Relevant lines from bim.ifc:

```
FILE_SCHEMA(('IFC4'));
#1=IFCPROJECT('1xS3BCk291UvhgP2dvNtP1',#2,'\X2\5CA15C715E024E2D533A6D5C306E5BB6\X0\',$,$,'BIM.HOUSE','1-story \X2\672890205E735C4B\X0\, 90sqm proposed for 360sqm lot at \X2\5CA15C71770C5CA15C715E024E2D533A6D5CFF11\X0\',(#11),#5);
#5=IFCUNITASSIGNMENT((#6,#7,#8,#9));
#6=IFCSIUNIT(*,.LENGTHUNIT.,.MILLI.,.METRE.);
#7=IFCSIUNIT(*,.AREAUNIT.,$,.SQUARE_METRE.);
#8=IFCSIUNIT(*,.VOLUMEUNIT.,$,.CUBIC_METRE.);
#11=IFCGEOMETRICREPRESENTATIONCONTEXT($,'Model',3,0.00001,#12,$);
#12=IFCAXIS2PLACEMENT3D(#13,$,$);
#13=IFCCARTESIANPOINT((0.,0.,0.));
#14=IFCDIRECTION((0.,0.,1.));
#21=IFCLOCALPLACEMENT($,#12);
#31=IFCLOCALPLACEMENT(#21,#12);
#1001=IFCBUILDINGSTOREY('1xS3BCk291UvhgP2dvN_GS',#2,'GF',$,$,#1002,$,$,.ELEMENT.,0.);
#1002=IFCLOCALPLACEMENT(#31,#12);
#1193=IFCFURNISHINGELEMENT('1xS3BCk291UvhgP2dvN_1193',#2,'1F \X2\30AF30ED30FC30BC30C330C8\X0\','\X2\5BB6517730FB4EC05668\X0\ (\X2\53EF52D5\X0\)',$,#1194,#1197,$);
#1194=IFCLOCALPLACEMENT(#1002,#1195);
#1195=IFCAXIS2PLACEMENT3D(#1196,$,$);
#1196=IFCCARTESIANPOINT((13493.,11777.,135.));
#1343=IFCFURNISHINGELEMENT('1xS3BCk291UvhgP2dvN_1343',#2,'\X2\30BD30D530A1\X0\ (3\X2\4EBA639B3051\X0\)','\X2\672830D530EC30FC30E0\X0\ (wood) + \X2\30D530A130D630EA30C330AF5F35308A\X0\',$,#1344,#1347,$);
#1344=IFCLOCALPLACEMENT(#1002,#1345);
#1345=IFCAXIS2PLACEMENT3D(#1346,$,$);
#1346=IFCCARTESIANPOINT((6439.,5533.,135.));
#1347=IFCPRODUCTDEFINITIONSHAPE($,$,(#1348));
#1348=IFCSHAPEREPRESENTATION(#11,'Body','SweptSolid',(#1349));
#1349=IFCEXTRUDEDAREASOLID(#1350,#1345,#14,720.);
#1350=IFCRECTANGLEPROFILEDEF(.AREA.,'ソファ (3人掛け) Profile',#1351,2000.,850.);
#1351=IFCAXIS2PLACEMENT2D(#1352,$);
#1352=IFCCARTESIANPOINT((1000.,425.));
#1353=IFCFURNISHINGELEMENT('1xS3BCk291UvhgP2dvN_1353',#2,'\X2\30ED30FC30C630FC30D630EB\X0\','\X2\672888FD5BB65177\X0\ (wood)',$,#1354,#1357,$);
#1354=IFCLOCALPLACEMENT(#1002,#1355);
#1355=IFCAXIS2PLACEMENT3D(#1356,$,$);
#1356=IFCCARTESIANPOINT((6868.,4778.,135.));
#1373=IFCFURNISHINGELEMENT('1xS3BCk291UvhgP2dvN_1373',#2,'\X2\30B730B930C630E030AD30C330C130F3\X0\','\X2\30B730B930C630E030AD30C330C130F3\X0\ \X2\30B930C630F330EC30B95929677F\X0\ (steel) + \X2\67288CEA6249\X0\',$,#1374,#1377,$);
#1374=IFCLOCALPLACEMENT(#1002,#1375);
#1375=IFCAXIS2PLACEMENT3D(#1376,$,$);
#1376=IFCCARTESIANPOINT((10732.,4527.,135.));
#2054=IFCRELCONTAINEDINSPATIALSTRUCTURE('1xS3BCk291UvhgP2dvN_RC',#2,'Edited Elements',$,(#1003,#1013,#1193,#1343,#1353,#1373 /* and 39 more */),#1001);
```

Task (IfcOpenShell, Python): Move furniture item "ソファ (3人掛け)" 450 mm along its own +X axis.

```python
import ifcopenshell
import ifcopenshell.api.geometry
import ifcopenshell.util.placement
import ifcopenshell.util.unit

model = ifcopenshell.open("bim.ifc")
unit_scale = ifcopenshell.util.unit.calculate_unit_scale(model)

item = model.by_id(1343)
matrix = ifcopenshell.util.placement.get_local_placement(item.ObjectPlacement)
matrix[:3, 3] += matrix[:3, 0] * 0.45 / unit_scale
ifcopenshell.api.geometry.edit_object_placement(model, product=item, matrix=matrix, is_si=False)

print(ifcopenshell.util.placement.get_local_placement(item.ObjectPlacement).round(3) + 0.0)

model.write("bim_rev.ifc")
```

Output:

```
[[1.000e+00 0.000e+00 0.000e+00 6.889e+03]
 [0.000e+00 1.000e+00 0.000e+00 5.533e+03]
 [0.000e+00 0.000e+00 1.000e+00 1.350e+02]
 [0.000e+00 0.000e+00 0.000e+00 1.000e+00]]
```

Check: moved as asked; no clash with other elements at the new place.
